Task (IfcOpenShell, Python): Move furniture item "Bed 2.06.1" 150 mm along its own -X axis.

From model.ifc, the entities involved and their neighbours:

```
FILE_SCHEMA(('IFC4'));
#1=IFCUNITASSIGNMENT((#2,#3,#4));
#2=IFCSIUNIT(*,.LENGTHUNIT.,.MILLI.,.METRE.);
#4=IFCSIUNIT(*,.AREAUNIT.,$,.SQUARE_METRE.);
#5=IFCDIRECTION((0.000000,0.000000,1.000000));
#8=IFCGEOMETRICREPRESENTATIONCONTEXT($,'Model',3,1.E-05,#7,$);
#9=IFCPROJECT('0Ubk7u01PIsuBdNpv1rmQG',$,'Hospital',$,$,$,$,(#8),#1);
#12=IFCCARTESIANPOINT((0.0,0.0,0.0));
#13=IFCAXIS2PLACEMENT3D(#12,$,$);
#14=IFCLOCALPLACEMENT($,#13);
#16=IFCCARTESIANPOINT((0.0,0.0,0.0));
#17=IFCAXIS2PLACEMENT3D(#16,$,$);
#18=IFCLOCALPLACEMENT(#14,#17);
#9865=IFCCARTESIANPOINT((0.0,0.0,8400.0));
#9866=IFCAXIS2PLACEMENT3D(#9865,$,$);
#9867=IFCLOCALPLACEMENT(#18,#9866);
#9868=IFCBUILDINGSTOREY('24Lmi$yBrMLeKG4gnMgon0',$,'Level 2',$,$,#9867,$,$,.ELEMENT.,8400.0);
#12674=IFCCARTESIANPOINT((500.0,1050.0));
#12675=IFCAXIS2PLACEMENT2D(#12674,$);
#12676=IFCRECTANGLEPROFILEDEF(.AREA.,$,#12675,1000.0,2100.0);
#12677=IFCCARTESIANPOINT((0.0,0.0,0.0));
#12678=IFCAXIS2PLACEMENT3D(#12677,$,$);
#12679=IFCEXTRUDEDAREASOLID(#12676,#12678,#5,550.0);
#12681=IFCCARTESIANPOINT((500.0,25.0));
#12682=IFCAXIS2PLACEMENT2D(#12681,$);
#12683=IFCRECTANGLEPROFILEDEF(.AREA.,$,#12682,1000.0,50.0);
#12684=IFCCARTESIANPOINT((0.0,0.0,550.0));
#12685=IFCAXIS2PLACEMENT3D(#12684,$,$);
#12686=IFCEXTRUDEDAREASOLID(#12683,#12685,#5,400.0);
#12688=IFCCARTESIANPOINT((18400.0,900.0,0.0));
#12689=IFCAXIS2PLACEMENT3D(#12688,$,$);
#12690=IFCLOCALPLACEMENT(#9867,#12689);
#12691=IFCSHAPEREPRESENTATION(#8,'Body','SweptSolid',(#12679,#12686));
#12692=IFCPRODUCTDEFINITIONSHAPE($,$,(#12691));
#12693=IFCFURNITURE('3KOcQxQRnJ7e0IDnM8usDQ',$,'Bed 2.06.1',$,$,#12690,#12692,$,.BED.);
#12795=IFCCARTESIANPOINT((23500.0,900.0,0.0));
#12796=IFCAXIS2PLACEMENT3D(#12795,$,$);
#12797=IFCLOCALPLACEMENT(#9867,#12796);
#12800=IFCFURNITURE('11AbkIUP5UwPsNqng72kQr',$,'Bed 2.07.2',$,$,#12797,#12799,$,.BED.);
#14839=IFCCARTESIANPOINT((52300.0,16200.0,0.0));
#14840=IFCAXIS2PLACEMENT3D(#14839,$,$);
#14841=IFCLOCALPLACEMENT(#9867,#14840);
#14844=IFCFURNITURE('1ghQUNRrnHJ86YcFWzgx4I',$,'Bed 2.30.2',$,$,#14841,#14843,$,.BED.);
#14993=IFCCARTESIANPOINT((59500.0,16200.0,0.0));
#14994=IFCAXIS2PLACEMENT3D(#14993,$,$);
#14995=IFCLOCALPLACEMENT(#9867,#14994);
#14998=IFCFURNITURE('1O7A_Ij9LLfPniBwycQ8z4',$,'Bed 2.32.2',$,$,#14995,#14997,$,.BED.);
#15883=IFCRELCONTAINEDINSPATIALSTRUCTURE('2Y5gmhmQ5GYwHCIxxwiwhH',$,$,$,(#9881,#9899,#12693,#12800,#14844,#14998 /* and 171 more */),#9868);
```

```python
import ifcopenshell
import ifcopenshell.api.geometry
import ifcopenshell.util.placement
import ifcopenshell.util.unit

model = ifcopenshell.open("model.ifc")
unit_scale = ifcopenshell.util.unit.calculate_unit_scale(model)

item = model.by_id(12693)
matrix = ifcopenshell.util.placement.get_local_placement(item.ObjectPlacement)
matrix[:3, 3] -= matrix[:3, 0] * 0.15 / unit_scale
ifcopenshell.api.geometry.edit_object_placement(model, product=item, matrix=matrix, is_si=False)

print(ifcopenshell.util.placement.get_local_placement(item.ObjectPlacement).round(3) + 0.0)

model.write("model_updated.ifc")
```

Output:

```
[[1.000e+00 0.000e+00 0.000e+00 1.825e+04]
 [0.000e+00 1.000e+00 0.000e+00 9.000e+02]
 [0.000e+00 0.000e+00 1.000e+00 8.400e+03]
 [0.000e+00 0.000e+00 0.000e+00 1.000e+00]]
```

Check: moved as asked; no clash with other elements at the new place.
